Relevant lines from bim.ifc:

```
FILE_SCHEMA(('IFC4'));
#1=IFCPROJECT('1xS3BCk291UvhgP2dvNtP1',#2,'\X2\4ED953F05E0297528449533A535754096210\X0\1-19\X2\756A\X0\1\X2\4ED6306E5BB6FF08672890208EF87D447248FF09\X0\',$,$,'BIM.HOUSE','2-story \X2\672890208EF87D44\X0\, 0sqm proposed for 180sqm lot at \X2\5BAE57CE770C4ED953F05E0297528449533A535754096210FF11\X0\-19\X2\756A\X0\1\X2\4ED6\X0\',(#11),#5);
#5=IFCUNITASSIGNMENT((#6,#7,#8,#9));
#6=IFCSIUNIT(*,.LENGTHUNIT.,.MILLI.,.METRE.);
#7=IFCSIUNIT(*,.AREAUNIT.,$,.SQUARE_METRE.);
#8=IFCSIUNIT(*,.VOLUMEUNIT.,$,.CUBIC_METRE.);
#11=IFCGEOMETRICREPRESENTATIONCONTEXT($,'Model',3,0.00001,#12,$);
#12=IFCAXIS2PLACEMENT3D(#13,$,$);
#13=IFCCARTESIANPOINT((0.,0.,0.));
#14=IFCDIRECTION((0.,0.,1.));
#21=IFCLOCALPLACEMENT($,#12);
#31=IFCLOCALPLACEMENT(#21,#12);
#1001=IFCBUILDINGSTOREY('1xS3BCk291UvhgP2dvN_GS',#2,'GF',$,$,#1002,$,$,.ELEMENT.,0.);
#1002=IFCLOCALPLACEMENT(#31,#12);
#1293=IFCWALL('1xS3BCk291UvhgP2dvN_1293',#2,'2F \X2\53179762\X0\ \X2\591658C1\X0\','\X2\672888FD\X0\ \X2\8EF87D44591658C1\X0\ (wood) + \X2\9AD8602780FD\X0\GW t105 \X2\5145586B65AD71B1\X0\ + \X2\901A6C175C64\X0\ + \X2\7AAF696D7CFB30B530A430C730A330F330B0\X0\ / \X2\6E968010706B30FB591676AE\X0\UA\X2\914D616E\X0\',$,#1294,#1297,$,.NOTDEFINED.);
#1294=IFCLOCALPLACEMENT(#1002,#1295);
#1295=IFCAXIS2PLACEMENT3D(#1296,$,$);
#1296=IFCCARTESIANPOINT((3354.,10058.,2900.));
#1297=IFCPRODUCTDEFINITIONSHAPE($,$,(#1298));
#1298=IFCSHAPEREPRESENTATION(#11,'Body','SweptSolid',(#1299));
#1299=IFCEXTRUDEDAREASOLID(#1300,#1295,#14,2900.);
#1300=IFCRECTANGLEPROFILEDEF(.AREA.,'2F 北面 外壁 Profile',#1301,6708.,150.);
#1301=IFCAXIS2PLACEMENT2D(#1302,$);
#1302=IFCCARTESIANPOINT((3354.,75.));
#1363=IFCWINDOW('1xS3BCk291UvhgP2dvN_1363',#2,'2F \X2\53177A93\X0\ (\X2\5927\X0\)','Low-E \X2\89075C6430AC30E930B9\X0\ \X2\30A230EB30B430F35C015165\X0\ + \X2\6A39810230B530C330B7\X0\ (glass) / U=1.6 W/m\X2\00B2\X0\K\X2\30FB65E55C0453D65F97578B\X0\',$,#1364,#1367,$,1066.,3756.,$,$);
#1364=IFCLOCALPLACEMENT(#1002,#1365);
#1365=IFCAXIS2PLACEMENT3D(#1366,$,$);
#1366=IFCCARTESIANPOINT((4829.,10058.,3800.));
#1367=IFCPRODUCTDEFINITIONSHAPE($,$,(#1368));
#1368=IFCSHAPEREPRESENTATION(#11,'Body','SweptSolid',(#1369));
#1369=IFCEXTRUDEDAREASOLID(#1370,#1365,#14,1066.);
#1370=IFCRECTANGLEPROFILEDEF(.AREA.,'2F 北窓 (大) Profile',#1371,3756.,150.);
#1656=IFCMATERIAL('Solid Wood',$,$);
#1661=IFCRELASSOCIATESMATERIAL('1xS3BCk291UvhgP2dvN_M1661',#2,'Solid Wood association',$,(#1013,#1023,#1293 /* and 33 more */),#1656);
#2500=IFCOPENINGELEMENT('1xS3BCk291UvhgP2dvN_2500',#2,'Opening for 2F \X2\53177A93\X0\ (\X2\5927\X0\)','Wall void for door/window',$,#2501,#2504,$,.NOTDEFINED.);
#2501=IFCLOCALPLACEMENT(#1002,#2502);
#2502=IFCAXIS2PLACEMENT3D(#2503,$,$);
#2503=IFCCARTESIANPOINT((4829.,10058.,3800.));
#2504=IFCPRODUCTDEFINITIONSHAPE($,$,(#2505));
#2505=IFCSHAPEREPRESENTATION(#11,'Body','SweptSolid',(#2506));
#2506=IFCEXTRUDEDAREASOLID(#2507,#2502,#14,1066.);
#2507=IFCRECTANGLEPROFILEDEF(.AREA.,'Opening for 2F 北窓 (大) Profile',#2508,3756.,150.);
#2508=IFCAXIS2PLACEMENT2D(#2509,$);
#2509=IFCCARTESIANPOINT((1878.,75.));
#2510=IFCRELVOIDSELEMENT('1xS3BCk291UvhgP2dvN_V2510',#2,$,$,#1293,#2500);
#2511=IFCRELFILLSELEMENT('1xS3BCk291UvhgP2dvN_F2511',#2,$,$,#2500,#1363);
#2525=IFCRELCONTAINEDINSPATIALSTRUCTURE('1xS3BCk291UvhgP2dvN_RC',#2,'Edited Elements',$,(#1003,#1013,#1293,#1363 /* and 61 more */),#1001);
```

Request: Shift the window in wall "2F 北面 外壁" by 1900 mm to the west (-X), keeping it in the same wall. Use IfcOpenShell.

```python
import ifcopenshell
import ifcopenshell.api.geometry
import ifcopenshell.util.placement

model = ifcopenshell.open("bim.ifc")

window = model.by_guid("1xS3BCk291UvhgP2dvN_1363")
opening = window.FillsVoids[0].RelatingOpeningElement
wall = opening.VoidsElements[0].RelatingBuildingElement

wall_matrix = ifcopenshell.util.placement.get_local_placement(wall.ObjectPlacement)
shift = wall_matrix[:3, 0] * -1900.0
before = ifcopenshell.util.placement.get_local_placement(window.ObjectPlacement)[:3, 3].copy()

# The window is not placed relative to its opening, so move both.
for product in (opening, window):
    matrix = ifcopenshell.util.placement.get_local_placement(product.ObjectPlacement)
    matrix[:3, 3] += shift
    ifcopenshell.api.geometry.edit_object_placement(model, product=product, matrix=matrix, is_si=False)

after = ifcopenshell.util.placement.get_local_placement(window.ObjectPlacement)[:3, 3]
print("window moved by", (after - before).round(3) + 0.0)

model.write("bim_edited.ifc")
```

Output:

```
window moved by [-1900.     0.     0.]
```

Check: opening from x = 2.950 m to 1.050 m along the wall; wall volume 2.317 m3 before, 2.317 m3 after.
